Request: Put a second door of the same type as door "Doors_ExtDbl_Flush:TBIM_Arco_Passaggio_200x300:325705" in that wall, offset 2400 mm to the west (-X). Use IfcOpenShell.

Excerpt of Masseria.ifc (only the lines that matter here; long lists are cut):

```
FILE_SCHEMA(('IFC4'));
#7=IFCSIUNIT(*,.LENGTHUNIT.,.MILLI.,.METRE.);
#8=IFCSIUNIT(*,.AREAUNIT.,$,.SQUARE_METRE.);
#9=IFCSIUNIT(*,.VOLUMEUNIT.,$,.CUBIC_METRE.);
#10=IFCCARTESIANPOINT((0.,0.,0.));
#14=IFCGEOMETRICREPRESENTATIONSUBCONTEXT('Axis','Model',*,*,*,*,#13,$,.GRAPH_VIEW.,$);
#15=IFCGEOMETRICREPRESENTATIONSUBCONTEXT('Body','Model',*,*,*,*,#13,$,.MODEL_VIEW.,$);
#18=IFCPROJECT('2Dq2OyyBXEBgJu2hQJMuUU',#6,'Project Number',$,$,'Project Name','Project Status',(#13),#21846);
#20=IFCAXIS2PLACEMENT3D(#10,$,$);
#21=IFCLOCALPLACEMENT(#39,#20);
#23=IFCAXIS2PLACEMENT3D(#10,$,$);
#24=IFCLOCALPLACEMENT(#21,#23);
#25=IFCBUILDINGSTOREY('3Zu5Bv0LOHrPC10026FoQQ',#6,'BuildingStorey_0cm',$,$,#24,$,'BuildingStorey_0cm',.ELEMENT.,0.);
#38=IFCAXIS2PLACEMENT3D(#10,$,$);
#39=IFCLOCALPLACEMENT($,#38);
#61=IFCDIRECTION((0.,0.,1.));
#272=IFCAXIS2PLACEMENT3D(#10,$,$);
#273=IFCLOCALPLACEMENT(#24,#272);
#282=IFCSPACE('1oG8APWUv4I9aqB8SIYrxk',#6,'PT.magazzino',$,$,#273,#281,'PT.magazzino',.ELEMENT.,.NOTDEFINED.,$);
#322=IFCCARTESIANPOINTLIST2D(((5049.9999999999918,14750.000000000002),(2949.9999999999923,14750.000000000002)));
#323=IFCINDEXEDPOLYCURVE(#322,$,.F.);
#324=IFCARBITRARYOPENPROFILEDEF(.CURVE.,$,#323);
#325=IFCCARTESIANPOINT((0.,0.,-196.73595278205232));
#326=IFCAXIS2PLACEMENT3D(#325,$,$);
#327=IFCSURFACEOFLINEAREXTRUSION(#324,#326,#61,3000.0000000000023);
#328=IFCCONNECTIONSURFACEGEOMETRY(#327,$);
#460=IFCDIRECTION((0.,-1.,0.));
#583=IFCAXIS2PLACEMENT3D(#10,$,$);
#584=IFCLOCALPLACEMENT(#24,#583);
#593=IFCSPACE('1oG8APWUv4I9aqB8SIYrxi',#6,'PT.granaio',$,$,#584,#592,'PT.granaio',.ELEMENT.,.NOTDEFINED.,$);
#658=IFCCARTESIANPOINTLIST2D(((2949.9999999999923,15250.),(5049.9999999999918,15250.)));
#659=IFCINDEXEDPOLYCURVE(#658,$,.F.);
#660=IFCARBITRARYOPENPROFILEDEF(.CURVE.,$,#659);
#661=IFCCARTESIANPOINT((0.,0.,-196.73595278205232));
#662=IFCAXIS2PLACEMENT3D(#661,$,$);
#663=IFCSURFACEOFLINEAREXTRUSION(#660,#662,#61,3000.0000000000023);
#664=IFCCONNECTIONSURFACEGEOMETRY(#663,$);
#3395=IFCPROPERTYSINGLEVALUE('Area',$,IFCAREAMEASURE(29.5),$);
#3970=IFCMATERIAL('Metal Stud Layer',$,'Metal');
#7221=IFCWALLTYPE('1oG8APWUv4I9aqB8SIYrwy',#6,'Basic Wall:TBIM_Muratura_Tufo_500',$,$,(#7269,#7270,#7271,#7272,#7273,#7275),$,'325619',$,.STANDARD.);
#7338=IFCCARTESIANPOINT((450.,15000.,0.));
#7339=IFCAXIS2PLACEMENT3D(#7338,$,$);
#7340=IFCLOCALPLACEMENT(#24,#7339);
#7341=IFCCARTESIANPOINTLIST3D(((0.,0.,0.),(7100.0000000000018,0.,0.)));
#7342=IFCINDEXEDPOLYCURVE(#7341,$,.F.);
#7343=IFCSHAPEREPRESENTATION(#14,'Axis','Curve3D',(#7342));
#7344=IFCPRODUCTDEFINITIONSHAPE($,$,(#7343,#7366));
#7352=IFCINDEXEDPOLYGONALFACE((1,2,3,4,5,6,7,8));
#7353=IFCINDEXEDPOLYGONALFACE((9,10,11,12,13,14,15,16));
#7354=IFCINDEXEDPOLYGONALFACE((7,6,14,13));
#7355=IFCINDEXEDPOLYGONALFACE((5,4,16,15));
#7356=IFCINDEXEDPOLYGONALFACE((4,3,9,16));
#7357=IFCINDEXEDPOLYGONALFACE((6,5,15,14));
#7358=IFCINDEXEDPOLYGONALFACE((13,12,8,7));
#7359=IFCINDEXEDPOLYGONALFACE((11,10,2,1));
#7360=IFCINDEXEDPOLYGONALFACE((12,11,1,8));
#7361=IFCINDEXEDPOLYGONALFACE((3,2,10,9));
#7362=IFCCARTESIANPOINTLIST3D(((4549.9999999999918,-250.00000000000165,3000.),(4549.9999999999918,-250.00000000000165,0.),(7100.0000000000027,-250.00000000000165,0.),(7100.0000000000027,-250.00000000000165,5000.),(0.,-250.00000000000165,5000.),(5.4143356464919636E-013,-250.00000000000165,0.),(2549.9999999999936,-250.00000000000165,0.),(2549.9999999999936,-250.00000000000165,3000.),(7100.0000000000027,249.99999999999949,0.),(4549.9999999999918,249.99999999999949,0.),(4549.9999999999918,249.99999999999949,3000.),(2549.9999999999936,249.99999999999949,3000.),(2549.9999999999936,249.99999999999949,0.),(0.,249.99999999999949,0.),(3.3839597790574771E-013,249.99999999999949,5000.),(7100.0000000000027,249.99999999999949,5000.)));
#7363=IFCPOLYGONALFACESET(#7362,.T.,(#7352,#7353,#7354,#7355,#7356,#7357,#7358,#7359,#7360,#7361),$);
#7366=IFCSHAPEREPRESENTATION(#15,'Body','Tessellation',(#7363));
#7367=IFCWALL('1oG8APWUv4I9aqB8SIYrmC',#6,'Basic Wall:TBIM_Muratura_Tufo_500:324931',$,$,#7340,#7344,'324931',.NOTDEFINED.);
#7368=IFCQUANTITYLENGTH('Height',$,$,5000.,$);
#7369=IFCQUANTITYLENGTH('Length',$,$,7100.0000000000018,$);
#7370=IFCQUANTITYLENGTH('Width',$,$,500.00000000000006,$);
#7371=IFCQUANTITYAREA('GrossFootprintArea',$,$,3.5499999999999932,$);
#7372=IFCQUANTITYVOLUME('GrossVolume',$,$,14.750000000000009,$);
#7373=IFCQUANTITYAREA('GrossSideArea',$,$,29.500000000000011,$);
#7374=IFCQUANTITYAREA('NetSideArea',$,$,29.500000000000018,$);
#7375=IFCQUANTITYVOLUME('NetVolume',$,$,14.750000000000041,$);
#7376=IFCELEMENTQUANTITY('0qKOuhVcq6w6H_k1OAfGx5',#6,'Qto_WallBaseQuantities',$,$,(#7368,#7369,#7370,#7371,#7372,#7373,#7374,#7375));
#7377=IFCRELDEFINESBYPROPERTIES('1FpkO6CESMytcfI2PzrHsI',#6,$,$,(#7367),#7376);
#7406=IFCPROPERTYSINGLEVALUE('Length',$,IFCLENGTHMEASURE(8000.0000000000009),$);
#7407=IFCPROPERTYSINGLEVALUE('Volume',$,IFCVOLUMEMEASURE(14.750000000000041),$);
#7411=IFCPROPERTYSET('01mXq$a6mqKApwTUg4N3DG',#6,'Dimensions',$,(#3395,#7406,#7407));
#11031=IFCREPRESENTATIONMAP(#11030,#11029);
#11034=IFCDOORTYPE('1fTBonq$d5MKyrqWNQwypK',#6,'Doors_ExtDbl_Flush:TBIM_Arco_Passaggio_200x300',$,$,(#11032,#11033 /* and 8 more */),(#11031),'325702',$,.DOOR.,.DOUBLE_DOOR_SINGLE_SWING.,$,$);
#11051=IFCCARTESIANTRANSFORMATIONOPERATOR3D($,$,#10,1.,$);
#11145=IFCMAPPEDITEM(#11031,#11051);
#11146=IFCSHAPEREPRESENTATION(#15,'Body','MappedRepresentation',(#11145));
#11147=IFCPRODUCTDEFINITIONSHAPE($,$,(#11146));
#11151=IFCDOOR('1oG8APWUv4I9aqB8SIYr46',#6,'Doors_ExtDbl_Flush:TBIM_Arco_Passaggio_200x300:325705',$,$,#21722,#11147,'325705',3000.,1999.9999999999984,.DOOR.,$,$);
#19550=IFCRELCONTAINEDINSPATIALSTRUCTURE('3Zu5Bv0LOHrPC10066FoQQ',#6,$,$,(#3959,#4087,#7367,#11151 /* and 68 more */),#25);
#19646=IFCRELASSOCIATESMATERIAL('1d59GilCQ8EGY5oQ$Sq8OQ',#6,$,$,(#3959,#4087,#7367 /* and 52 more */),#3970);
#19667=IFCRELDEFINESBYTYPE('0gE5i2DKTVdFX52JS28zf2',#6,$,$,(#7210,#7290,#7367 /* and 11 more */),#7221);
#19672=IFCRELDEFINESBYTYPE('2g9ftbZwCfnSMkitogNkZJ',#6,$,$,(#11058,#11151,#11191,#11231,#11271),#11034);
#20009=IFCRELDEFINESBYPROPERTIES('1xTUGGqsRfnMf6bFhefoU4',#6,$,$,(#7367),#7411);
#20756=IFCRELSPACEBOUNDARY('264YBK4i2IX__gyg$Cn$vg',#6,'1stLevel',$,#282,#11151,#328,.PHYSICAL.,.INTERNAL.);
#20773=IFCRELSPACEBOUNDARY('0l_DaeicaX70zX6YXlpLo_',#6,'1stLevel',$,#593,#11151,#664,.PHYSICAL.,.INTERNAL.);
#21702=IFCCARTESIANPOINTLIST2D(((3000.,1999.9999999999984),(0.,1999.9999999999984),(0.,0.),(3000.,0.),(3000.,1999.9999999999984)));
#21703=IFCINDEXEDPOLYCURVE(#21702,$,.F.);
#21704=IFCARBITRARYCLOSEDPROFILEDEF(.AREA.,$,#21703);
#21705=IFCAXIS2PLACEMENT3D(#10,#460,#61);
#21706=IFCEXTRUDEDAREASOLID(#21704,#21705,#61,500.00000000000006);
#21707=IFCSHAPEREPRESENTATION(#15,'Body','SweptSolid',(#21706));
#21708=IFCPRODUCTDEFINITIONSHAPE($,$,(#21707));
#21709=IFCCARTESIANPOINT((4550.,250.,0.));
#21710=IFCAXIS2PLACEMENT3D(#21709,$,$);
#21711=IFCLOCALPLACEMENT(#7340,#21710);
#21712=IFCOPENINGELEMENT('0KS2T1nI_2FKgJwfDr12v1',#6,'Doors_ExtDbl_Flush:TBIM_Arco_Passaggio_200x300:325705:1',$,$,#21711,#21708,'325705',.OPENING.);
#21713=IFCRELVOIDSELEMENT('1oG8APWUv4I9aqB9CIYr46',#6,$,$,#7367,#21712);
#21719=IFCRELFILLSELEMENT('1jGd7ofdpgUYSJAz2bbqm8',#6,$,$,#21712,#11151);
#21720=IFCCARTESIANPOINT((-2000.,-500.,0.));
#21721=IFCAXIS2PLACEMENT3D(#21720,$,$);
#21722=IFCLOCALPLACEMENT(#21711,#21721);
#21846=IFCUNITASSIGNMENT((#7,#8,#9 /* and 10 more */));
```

```python
import numpy as np
import ifcopenshell
import ifcopenshell.api.feature
import ifcopenshell.api.geometry
import ifcopenshell.api.pset
import ifcopenshell.api.root
import ifcopenshell.geom
import ifcopenshell.util.element
import ifcopenshell.util.placement
import ifcopenshell.util.shape
import ifcopenshell.util.unit

model = ifcopenshell.open("Masseria.ifc")
area_scale = ifcopenshell.util.unit.calculate_unit_scale(model, "AREAUNIT")
volume_scale = ifcopenshell.util.unit.calculate_unit_scale(model, "VOLUMEUNIT")
settings = ifcopenshell.geom.settings()


def volume(element):
    """Net volume in cubic metres, openings subtracted."""
    shape = ifcopenshell.geom.create_shape(settings, element)
    return ifcopenshell.util.shape.get_volume(shape.geometry)


def reuse_history(source, copy):
    """copy_class also copies each property set's owner history, people and application; keep the originals."""
    for rel in copy.IsDefinedBy:
        if rel.is_a("IfcRelDefinesByProperties") and (history := rel.RelatingPropertyDefinition.OwnerHistory):
            rel.RelatingPropertyDefinition.OwnerHistory = source.OwnerHistory
            ifcopenshell.util.element.remove_deep2(model, history)


door = model.by_guid("1oG8APWUv4I9aqB8SIYr46")
opening = door.FillsVoids[0].RelatingOpeningElement
wall = opening.VoidsElements[0].RelatingBuildingElement
before = volume(wall)
shift = ifcopenshell.util.placement.get_local_placement(wall.ObjectPlacement)[:3, 0] * -2400.0

# copy_class copies the void relationship, type, container and properties, but no geometry.
new_opening = ifcopenshell.api.root.copy_class(model, product=opening)
new_opening.Representation = ifcopenshell.util.element.copy_deep(
    model, opening.Representation, exclude=["IfcGeometricRepresentationContext", "IfcRepresentationMap"]
)
new_opening.Name = "Doors_ExtDbl_Flush:TBIM_Arco_Passaggio_200x300"
new_opening.Tag = None
reuse_history(opening, new_opening)
new_door = ifcopenshell.api.root.copy_class(model, product=door)
new_door.Representation = ifcopenshell.util.element.copy_deep(
    model, door.Representation, exclude=["IfcGeometricRepresentationContext", "IfcRepresentationMap"]
)
new_door.Name = "Doors_ExtDbl_Flush:TBIM_Arco_Passaggio_200x300"
new_door.Tag = None
reuse_history(door, new_door)
ifcopenshell.api.feature.add_filling(model, opening=new_opening, element=new_door)

for old, new in ((opening, new_opening), (door, new_door)):
    matrix = ifcopenshell.util.placement.get_local_placement(old.ObjectPlacement)
    matrix[:3, 3] += shift
    ifcopenshell.api.geometry.edit_object_placement(model, product=new, matrix=matrix, is_si=False)

# The copied space boundaries still share their surfaces with the original.
for rel in new_door.ProvidesBoundaries:
    if rel.ConnectionGeometry:
        rel.ConnectionGeometry = ifcopenshell.util.element.copy_deep(model, rel.ConnectionGeometry)

# Space boundary surfaces are stored in each space's coordinates; move them too.
for rel in new_door.ProvidesBoundaries:
    if not rel.ConnectionGeometry:
        continue
    surface = rel.ConnectionGeometry.SurfaceOnRelatingElement
    space_matrix = ifcopenshell.util.placement.get_local_placement(rel.RelatingSpace.ObjectPlacement)
    point = np.array(surface.Position.Location.Coordinates) + space_matrix[:3, :3].T @ shift
    surface.Position = model.createIfcAxis2Placement3D(
        model.createIfcCartesianPoint(point.tolist()), surface.Position.Axis, surface.Position.RefDirection
    )

after = volume(wall)
thickness = 0.5  # wall thickness in metres

# Update the wall's stored quantities.
qto = model.by_id(ifcopenshell.util.element.get_pset(wall, "Qto_WallBaseQuantities", should_inherit=False)["id"])
ifcopenshell.api.pset.edit_qto(model, qto=qto, properties={
    "NetSideArea": after / thickness / area_scale,
    "NetVolume": after / volume_scale,
})
pset = model.by_id(ifcopenshell.util.element.get_pset(wall, "Dimensions", should_inherit=False)["id"])
ifcopenshell.api.pset.edit_pset(model, pset=pset, properties={
    "Area": model.create_entity("IfcAreaMeasure", after / thickness / area_scale),
    "Volume": model.create_entity("IfcVolumeMeasure", after / volume_scale),
})

print(f"wall volume {before:.3f} -> {after:.3f} m3")

model.write("Masseria_rev.ifc")
```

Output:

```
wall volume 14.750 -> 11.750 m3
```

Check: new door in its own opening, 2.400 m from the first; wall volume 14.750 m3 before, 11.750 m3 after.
